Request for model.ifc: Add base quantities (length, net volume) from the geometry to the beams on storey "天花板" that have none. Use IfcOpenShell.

First a look at what the model holds.

```python
import ifcopenshell
import ifcopenshell.util.element
import ifcopenshell.util.unit

model = ifcopenshell.open("model.ifc")
print(model.schema)
for unit_type in ("LENGTHUNIT", "AREAUNIT", "VOLUMEUNIT"):
    print(unit_type, ifcopenshell.util.unit.calculate_unit_scale(model, unit_type))
storey = next(s for s in model.by_type("IfcBuildingStorey") if s.Name == "天花板")
beams = [e for e in ifcopenshell.util.element.get_decomposition(storey) if e.is_a("IfcBeam")]
for e in sorted(beams, key=lambda e: e.id()):
    print(e.id(), e.is_a(), e.Name, list(ifcopenshell.util.element.get_psets(e, qtos_only=True)), sep=" | ")
```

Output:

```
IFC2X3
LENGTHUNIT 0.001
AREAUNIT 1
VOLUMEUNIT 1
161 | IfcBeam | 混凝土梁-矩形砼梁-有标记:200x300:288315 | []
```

```python
import ifcopenshell
import ifcopenshell.api.pset
import ifcopenshell.geom
import ifcopenshell.util.element
import ifcopenshell.util.shape
import ifcopenshell.util.unit

model = ifcopenshell.open("model.ifc")
unit_scale = ifcopenshell.util.unit.calculate_unit_scale(model)
volume_scale = ifcopenshell.util.unit.calculate_unit_scale(model, "VOLUMEUNIT")
settings = ifcopenshell.geom.settings()

storey = next(s for s in model.by_type("IfcBuildingStorey") if s.Name == "天花板")
beams = [e for e in ifcopenshell.util.element.get_decomposition(storey) if e.is_a("IfcBeam")]

for e in sorted(beams, key=lambda e: e.id()):
    if ifcopenshell.util.element.get_psets(e, qtos_only=True, should_inherit=False):
        continue
    # Geometry comes back in metres, in the element's own axes.
    shape = ifcopenshell.geom.create_shape(settings, e)
    values = {
        "Length": ifcopenshell.util.shape.get_max_xyz(shape.geometry) / unit_scale,
        "NetVolume": ifcopenshell.util.shape.get_volume(shape.geometry) / volume_scale,
    }
    qto = ifcopenshell.api.pset.add_qto(model, product=e, name="BaseQuantities")
    ifcopenshell.api.pset.edit_qto(model, qto=qto, properties=values)
    print(e.id(), {k: round(v, 3) for k, v in values.items()})

model.write("model_edited.ifc")
```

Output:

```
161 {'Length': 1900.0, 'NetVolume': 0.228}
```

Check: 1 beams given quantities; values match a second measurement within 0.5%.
